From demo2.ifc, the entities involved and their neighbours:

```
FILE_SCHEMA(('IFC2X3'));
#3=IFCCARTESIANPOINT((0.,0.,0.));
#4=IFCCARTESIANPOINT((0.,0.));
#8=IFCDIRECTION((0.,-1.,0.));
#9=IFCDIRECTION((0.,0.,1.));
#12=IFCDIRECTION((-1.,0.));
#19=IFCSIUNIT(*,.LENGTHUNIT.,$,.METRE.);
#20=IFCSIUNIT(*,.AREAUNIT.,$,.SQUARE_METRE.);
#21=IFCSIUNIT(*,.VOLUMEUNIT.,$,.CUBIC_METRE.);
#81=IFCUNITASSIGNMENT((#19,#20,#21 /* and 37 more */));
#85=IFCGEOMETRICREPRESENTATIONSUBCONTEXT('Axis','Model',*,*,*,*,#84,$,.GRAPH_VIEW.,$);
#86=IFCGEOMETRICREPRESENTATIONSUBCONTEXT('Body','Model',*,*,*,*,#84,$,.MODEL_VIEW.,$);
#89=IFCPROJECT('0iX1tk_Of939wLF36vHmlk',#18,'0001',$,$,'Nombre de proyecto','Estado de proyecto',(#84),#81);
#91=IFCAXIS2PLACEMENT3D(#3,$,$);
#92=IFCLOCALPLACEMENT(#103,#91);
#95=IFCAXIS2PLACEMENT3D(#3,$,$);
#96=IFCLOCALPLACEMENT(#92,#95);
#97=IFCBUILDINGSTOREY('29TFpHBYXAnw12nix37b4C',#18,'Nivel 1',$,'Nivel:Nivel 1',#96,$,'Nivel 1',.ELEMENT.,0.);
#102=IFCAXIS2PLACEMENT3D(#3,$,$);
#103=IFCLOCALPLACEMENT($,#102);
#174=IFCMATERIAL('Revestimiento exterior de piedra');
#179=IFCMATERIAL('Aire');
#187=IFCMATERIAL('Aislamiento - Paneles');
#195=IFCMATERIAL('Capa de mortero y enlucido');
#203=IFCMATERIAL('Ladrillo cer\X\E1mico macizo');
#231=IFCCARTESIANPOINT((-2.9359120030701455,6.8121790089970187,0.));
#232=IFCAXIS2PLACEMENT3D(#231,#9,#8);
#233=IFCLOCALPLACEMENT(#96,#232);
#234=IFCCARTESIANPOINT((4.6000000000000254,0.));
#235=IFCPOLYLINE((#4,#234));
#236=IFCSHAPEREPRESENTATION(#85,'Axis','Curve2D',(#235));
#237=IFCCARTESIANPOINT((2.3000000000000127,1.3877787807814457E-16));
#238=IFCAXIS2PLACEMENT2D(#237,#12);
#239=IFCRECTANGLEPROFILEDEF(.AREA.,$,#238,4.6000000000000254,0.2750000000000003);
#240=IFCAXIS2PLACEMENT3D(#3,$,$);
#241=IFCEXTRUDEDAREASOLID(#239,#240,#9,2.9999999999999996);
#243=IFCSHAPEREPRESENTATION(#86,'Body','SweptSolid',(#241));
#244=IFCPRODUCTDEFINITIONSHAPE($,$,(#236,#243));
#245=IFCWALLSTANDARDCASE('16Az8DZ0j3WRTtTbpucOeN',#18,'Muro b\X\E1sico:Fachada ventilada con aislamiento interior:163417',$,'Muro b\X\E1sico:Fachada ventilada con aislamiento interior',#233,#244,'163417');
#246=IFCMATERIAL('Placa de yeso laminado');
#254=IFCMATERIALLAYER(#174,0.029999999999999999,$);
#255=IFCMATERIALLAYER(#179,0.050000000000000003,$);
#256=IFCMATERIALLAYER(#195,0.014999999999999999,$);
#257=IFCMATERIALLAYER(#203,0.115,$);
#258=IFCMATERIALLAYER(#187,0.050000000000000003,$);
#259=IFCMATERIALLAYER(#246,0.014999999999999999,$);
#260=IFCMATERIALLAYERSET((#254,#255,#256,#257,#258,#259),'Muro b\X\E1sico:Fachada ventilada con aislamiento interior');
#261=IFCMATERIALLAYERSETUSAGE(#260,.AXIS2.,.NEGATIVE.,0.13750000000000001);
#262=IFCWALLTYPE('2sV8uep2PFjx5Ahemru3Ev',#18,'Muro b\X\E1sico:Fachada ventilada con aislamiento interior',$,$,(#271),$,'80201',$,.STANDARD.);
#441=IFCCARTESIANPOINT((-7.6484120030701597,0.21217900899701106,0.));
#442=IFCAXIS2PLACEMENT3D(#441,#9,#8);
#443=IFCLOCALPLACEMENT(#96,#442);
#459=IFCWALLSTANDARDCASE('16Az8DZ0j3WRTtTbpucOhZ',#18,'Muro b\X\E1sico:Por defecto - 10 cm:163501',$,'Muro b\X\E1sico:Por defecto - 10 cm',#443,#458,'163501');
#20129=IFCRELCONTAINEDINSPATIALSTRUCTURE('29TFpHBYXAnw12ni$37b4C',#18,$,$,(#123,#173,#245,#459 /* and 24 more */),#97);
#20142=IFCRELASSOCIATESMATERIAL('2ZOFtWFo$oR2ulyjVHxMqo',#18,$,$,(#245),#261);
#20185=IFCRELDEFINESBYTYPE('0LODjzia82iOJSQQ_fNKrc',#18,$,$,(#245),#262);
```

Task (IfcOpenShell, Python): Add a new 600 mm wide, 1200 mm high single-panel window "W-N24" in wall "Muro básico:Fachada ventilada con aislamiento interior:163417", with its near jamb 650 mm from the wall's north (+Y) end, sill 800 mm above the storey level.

```python
import numpy as np
import ifcopenshell
import ifcopenshell.api.feature
import ifcopenshell.api.geometry
import ifcopenshell.api.root
import ifcopenshell.api.spatial
import ifcopenshell.api.type
import ifcopenshell.geom
import ifcopenshell.util.element
import ifcopenshell.util.placement
import ifcopenshell.util.representation
import ifcopenshell.util.shape
import ifcopenshell.util.unit

model = ifcopenshell.open("demo2.ifc")
unit_scale = ifcopenshell.util.unit.calculate_unit_scale(model)
settings = ifcopenshell.geom.settings()


def volume(element):
    """Net volume in cubic metres, openings subtracted."""
    shape = ifcopenshell.geom.create_shape(settings, element)
    return ifcopenshell.util.shape.get_volume(shape.geometry)


wall = model.by_guid("16Az8DZ0j3WRTtTbpucOeN")
storey = ifcopenshell.util.element.get_container(wall, ifc_class="IfcBuildingStorey")
context = ifcopenshell.util.representation.get_context(model, "Model", "Body", "MODEL_VIEW")
before = volume(wall)

width, height, from_end, sill = 0.6, 1.2, 0.65, 0.8  # metres

# The wall runs along its own X axis, and the end named is its -X end.
wall_shape = ifcopenshell.geom.create_shape(settings, wall)
x, y, z = ifcopenshell.util.shape.get_vertices(wall_shape.geometry).T
start = x.min() + from_end
face, thickness = float(y.min()), float(y.max() - y.min())
wall_matrix = ifcopenshell.util.placement.get_local_placement(wall.ObjectPlacement)
level = ifcopenshell.util.placement.get_local_placement(storey.ObjectPlacement)[2, 3]


def in_wall(x, y):
    """Placement at x, y metres in the wall's axes, at sill height."""
    matrix = wall_matrix.copy()
    matrix[:, 3] = wall_matrix @ np.array([x / unit_scale, y / unit_scale, 0.0, 1.0])
    matrix[2, 3] = level + sill / unit_scale
    return matrix


# Opening: a box that overshoots both wall faces by 50 mm.
opening = ifcopenshell.api.root.create_entity(model, ifc_class="IfcOpeningElement")
box = ifcopenshell.api.geometry.add_wall_representation(
    model, context=context, length=width, height=height, thickness=thickness + 0.1
)
ifcopenshell.api.geometry.assign_representation(model, product=opening, representation=box)
ifcopenshell.api.geometry.edit_object_placement(model, product=opening, matrix=in_wall(start, face - 0.05), is_si=False)
ifcopenshell.api.feature.add_feature(model, feature=opening, element=wall)

window = ifcopenshell.api.root.create_entity(model, ifc_class="IfcWindow", name="W-N24")
window.OverallWidth, window.OverallHeight = width / unit_scale, height / unit_scale
body = ifcopenshell.api.geometry.add_window_representation(
    model,
    context=context,
    overall_width=window.OverallWidth,
    overall_height=window.OverallHeight,
    partition_type="SINGLE_PANEL",
)
ifcopenshell.api.geometry.assign_representation(model, product=window, representation=body)
ifcopenshell.api.spatial.assign_container(model, products=[window], relating_structure=storey)
fills = ifcopenshell.api.feature.add_filling(model, opening=opening, element=window)
fills.OwnerHistory = window.OwnerHistory  # required in IFC2X3

# IFC2X3 keeps the operation on the window style.
style = ifcopenshell.api.root.create_entity(model, ifc_class="IfcWindowStyle", name="W-N24")
style.OperationType, style.ConstructionType = "SINGLE_PANEL", "NOTDEFINED"
style.ParameterTakesPrecedence = style.Sizeable = False
ifcopenshell.api.type.assign_type(model, related_objects=[window], relating_type=style)

# Centre the window in the wall's thickness.
ifcopenshell.api.geometry.edit_object_placement(model, product=window, matrix=in_wall(start, face), is_si=False)
window_shape = ifcopenshell.geom.create_shape(settings, window)
depth = ifcopenshell.util.shape.get_vertices(window_shape.geometry)[:, 1]
offset = face + thickness / 2 - (depth.min() + depth.max()) / 2
ifcopenshell.api.geometry.edit_object_placement(model, product=window, matrix=in_wall(start, offset), is_si=False)

after = volume(wall)

print(f"wall volume {before:.3f} -> {after:.3f} m3")

model.write("demo2_updated.ifc")
```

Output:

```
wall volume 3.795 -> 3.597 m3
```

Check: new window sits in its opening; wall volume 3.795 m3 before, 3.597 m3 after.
